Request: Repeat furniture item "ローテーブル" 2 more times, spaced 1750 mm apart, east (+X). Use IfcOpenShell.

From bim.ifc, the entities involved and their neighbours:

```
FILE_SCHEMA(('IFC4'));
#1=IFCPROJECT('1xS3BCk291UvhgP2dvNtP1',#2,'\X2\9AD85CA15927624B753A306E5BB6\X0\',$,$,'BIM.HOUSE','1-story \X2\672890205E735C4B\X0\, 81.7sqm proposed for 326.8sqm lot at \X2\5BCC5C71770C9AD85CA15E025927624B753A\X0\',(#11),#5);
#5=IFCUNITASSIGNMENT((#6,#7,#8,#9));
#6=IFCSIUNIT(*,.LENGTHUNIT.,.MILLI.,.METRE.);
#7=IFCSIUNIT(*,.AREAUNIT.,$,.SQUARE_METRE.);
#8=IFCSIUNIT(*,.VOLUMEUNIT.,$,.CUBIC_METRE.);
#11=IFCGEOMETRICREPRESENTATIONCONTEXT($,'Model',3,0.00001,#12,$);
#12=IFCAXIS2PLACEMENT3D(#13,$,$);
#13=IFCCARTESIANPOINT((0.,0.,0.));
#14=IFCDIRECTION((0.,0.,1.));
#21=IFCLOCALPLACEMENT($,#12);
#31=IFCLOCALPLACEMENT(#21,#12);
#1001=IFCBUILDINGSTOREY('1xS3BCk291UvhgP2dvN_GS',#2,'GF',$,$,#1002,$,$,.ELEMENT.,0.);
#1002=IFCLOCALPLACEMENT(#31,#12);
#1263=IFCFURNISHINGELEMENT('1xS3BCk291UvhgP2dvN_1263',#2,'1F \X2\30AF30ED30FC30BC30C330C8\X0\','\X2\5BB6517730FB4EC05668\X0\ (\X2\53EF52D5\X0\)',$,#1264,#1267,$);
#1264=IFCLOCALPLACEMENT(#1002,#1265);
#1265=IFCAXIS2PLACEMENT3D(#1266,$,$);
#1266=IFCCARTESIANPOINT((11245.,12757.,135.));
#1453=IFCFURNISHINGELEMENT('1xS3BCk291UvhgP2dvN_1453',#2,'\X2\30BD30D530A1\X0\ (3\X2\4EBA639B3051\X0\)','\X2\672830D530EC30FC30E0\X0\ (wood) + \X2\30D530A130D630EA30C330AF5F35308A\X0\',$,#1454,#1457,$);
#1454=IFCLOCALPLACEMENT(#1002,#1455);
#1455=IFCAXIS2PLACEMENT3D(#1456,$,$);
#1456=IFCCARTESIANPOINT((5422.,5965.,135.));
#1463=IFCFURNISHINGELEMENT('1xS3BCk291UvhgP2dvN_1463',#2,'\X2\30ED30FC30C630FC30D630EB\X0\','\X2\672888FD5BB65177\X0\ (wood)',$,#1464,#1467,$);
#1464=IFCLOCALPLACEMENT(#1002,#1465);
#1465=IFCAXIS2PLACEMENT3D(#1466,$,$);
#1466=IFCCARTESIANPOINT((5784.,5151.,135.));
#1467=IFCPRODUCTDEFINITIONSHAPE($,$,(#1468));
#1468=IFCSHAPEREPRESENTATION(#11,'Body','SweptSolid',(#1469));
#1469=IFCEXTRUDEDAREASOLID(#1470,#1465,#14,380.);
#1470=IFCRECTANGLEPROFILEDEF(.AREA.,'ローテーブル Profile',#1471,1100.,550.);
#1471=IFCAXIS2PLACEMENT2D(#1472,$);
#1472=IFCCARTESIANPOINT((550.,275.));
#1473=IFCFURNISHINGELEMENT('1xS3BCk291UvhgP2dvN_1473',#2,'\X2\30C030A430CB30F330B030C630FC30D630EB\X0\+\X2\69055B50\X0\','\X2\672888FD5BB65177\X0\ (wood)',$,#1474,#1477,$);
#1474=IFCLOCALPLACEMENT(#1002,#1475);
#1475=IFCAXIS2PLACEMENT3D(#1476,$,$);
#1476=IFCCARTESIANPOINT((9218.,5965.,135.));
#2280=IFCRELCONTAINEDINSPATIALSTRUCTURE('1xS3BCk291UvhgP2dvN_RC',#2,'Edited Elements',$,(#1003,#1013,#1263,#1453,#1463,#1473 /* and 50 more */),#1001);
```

```python
import numpy as np
import ifcopenshell
import ifcopenshell.api.geometry
import ifcopenshell.api.root
import ifcopenshell.util.element
import ifcopenshell.util.placement
import ifcopenshell.util.unit

model = ifcopenshell.open("bim.ifc")
unit_scale = ifcopenshell.util.unit.calculate_unit_scale(model)


def reuse_history(source, copy):
    """copy_class also copies each property set's owner history, people and application; keep the originals."""
    for rel in copy.IsDefinedBy:
        if rel.is_a("IfcRelDefinesByProperties") and (history := rel.RelatingPropertyDefinition.OwnerHistory):
            rel.RelatingPropertyDefinition.OwnerHistory = source.OwnerHistory
            ifcopenshell.util.element.remove_deep2(model, history)


source = model.by_id(1463)
base = ifcopenshell.util.placement.get_local_placement(source.ObjectPlacement)
step = np.array([1.0, 0.0, 0.0]) * 1.75 / unit_scale

for i in range(1, 3):
    copy = ifcopenshell.api.root.copy_class(model, product=source)
    copy.Representation = ifcopenshell.util.element.copy_deep(
        model, source.Representation, exclude=["IfcGeometricRepresentationContext", "IfcRepresentationMap"]
    )
    reuse_history(source, copy)
    matrix = base.copy()
    matrix[:3, 3] += i * step
    print("added at", matrix[:3, 3].round(3) + 0.0)
    ifcopenshell.api.geometry.edit_object_placement(model, product=copy, matrix=matrix, is_si=False)

model.write("bim_v2.ifc")
```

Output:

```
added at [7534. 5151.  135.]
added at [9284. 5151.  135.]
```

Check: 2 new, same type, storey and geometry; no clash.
